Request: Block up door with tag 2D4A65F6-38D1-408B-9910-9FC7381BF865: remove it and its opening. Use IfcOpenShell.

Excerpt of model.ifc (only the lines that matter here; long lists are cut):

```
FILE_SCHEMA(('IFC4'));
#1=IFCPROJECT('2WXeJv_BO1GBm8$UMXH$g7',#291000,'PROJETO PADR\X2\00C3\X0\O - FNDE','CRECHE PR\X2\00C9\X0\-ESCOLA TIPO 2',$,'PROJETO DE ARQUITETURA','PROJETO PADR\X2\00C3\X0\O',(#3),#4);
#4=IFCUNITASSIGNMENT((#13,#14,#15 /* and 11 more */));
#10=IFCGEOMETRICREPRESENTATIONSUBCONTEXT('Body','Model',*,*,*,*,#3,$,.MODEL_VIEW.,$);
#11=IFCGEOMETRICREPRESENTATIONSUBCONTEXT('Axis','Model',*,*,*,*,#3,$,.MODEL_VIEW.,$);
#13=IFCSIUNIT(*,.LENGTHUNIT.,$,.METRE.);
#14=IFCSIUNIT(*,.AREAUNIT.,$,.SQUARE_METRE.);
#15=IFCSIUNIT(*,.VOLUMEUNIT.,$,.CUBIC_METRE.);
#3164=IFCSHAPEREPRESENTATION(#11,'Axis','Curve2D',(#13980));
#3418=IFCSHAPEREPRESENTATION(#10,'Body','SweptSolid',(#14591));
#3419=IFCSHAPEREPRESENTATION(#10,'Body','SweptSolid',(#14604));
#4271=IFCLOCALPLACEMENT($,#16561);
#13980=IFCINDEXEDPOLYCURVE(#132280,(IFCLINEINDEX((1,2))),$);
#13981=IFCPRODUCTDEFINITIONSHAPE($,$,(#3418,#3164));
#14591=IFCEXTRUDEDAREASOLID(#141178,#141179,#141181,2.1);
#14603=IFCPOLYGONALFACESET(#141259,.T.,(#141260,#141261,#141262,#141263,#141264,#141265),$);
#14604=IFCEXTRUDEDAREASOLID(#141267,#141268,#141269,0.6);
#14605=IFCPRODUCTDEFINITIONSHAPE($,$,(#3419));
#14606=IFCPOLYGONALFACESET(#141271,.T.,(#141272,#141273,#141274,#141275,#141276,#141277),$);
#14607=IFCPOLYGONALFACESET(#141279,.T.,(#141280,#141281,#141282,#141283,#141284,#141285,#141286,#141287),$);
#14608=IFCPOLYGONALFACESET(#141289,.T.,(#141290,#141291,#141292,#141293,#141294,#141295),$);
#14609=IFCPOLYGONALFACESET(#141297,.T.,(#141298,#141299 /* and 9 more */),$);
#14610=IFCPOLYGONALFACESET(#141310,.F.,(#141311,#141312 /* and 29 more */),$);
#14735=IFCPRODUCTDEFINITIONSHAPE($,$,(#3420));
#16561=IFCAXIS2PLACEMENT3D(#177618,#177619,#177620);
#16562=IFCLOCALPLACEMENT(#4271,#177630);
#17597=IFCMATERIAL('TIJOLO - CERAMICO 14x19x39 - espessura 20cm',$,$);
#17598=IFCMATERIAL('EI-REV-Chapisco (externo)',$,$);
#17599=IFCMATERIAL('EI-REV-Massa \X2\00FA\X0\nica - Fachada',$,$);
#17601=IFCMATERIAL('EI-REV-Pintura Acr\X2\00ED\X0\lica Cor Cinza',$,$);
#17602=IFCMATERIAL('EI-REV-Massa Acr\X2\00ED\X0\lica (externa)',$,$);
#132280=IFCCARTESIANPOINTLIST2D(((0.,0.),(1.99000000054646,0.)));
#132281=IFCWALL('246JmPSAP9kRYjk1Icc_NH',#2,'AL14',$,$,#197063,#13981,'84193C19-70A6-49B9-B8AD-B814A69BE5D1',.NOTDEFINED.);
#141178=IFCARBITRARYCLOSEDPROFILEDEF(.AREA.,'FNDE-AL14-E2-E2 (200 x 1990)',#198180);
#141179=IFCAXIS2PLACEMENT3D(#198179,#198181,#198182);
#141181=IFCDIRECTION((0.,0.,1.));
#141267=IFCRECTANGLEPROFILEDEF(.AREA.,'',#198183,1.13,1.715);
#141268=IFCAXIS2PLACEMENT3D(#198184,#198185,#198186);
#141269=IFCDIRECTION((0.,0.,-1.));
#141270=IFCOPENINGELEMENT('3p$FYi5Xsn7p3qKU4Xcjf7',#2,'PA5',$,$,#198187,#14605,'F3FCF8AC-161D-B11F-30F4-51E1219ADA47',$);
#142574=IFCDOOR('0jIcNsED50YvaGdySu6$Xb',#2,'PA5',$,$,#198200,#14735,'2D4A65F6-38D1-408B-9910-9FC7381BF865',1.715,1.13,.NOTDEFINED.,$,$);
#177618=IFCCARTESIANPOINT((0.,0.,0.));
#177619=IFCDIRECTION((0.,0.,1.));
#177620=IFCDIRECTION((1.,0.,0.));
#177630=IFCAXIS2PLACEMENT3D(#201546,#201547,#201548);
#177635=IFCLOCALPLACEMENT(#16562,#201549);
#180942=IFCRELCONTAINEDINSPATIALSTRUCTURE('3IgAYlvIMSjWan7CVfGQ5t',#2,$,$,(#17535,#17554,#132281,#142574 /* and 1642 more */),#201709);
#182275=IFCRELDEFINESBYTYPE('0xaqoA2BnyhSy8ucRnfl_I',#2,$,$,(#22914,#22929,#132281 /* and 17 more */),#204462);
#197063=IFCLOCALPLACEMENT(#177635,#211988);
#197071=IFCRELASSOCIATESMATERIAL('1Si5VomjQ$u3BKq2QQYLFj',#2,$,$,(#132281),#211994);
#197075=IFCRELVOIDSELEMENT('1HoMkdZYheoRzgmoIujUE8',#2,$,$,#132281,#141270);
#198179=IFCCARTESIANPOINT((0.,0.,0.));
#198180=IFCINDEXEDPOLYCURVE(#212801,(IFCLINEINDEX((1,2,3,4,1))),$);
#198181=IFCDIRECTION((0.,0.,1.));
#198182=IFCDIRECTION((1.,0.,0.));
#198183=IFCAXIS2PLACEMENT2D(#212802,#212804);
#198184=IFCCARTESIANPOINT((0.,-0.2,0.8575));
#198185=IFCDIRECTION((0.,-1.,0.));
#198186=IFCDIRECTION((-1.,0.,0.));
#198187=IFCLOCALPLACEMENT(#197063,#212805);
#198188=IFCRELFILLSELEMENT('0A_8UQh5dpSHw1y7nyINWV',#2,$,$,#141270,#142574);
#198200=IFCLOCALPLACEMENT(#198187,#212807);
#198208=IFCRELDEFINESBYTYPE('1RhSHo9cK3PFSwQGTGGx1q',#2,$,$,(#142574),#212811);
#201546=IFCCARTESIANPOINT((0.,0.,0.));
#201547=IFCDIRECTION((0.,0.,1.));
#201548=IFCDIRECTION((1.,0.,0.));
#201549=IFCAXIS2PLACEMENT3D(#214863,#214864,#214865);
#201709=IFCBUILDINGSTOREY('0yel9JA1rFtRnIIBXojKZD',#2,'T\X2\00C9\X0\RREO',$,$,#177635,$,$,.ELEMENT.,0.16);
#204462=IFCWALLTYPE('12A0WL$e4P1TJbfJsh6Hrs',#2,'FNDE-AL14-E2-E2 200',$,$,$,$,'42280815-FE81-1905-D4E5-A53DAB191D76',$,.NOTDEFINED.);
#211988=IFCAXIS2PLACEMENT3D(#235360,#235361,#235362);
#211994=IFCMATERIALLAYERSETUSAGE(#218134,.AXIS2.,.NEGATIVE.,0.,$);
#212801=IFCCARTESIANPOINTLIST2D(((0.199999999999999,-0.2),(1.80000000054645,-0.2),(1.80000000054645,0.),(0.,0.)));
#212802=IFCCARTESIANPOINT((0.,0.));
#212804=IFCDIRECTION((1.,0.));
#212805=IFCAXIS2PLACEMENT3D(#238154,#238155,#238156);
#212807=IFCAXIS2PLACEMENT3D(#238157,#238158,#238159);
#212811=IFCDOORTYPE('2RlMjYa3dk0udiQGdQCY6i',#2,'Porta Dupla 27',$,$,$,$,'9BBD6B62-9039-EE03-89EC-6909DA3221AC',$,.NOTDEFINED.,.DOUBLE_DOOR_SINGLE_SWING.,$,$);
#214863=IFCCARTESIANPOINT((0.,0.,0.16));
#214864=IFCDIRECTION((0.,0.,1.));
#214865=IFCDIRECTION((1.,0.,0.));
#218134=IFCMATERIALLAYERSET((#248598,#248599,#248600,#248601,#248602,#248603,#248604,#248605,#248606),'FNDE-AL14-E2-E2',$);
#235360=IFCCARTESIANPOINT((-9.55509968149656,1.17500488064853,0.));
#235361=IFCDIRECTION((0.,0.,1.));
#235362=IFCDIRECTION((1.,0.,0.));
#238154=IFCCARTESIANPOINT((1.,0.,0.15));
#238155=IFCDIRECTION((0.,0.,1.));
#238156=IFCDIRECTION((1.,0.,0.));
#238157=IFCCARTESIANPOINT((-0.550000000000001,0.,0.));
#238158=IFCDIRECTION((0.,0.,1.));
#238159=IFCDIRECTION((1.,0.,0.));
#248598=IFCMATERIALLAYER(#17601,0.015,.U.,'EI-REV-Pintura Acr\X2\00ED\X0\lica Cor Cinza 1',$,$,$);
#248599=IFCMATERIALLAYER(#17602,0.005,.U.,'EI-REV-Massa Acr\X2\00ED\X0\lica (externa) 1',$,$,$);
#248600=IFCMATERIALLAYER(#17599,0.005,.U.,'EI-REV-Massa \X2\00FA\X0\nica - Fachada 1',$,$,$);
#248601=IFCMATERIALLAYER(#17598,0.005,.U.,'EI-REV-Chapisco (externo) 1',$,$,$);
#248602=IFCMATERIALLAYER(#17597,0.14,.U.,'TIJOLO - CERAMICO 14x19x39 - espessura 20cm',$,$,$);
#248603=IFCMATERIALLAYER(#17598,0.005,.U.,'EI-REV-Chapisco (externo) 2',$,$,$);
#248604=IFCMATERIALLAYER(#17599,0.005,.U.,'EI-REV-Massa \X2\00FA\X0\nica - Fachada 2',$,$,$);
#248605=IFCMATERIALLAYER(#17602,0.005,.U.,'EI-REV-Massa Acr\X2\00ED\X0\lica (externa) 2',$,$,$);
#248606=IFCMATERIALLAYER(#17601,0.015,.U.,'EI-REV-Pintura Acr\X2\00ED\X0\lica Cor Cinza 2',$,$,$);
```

```python
import ifcopenshell
import ifcopenshell.api.feature
import ifcopenshell.api.root
import ifcopenshell.geom
import ifcopenshell.util.shape

model = ifcopenshell.open("model.ifc")
settings = ifcopenshell.geom.settings()


def volume(element):
    """Net volume in cubic metres, openings subtracted."""
    shape = ifcopenshell.geom.create_shape(settings, element)
    return ifcopenshell.util.shape.get_volume(shape.geometry)


door = model.by_guid("0jIcNsED50YvaGdySu6$Xb")
opening = door.FillsVoids[0].RelatingOpeningElement
wall = opening.VoidsElements[0].RelatingBuildingElement
before = volume(wall)

ifcopenshell.api.root.remove_product(model, product=door)
ifcopenshell.api.feature.remove_feature(model, feature=opening)

after = volume(wall)

print(f"wall volume {before:.3f} -> {after:.3f} m3")

model.write("model_updated.ifc")
```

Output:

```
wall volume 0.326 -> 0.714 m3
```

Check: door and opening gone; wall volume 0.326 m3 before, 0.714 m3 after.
